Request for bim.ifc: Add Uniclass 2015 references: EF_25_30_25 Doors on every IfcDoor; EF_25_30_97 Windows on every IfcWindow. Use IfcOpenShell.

First a look at what the model holds.

```python
import ifcopenshell

model = ifcopenshell.open("bim.ifc")
print(model.schema)
print("classifications:", [c.Name for c in model.by_type("IfcClassification")])
for ifc_class in ("IfcDoor", "IfcRoof", "IfcStair", "IfcWall", "IfcWindow"):
    print(ifc_class, len(model.by_type(ifc_class)))
```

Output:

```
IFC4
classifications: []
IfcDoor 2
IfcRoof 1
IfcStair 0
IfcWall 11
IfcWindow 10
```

```python
import ifcopenshell
import ifcopenshell.api.classification

model = ifcopenshell.open("bim.ifc")

system = ifcopenshell.api.classification.add_classification(model, classification="Uniclass 2015")

codes = {
    "IfcDoor": ("EF_25_30_25", "Doors"),
    "IfcWindow": ("EF_25_30_97", "Windows"),
}
for ifc_class, (code, name) in codes.items():
    products = model.by_type(ifc_class)
    ifcopenshell.api.classification.add_reference(
        model, products=products, classification=system, identification=code, name=name
    )
    print(code, len(products))

model.write("bim_updated.ifc")
```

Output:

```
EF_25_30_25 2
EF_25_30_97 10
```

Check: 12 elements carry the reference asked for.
